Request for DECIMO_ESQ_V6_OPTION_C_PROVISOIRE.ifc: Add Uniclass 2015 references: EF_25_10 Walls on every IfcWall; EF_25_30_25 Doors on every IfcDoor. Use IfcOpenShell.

First a look at what the model holds.

```python
import ifcopenshell

model = ifcopenshell.open("DECIMO_ESQ_V6_OPTION_C_PROVISOIRE.ifc")
print(model.schema)
print("classifications:", [c.Name for c in model.by_type("IfcClassification")])
for ifc_class in ("IfcDoor", "IfcRoof", "IfcStair", "IfcWall", "IfcWindow"):
    print(ifc_class, len(model.by_type(ifc_class)))
```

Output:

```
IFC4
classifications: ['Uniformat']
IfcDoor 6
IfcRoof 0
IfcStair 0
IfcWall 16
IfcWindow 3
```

```python
import ifcopenshell
import ifcopenshell.api.classification

model = ifcopenshell.open("DECIMO_ESQ_V6_OPTION_C_PROVISOIRE.ifc")

system = ifcopenshell.api.classification.add_classification(model, classification="Uniclass 2015")

codes = {
    "IfcWall": ("EF_25_10", "Walls"),
    "IfcDoor": ("EF_25_30_25", "Doors"),
}
for ifc_class, (code, name) in codes.items():
    products = model.by_type(ifc_class)
    ifcopenshell.api.classification.add_reference(
        model, products=products, classification=system, identification=code, name=name
    )
    print(code, len(products))

model.write("DECIMO_ESQ_V6_OPTION_C_PROVISOIRE_edited.ifc")
```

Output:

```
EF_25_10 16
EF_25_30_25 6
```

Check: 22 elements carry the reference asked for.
